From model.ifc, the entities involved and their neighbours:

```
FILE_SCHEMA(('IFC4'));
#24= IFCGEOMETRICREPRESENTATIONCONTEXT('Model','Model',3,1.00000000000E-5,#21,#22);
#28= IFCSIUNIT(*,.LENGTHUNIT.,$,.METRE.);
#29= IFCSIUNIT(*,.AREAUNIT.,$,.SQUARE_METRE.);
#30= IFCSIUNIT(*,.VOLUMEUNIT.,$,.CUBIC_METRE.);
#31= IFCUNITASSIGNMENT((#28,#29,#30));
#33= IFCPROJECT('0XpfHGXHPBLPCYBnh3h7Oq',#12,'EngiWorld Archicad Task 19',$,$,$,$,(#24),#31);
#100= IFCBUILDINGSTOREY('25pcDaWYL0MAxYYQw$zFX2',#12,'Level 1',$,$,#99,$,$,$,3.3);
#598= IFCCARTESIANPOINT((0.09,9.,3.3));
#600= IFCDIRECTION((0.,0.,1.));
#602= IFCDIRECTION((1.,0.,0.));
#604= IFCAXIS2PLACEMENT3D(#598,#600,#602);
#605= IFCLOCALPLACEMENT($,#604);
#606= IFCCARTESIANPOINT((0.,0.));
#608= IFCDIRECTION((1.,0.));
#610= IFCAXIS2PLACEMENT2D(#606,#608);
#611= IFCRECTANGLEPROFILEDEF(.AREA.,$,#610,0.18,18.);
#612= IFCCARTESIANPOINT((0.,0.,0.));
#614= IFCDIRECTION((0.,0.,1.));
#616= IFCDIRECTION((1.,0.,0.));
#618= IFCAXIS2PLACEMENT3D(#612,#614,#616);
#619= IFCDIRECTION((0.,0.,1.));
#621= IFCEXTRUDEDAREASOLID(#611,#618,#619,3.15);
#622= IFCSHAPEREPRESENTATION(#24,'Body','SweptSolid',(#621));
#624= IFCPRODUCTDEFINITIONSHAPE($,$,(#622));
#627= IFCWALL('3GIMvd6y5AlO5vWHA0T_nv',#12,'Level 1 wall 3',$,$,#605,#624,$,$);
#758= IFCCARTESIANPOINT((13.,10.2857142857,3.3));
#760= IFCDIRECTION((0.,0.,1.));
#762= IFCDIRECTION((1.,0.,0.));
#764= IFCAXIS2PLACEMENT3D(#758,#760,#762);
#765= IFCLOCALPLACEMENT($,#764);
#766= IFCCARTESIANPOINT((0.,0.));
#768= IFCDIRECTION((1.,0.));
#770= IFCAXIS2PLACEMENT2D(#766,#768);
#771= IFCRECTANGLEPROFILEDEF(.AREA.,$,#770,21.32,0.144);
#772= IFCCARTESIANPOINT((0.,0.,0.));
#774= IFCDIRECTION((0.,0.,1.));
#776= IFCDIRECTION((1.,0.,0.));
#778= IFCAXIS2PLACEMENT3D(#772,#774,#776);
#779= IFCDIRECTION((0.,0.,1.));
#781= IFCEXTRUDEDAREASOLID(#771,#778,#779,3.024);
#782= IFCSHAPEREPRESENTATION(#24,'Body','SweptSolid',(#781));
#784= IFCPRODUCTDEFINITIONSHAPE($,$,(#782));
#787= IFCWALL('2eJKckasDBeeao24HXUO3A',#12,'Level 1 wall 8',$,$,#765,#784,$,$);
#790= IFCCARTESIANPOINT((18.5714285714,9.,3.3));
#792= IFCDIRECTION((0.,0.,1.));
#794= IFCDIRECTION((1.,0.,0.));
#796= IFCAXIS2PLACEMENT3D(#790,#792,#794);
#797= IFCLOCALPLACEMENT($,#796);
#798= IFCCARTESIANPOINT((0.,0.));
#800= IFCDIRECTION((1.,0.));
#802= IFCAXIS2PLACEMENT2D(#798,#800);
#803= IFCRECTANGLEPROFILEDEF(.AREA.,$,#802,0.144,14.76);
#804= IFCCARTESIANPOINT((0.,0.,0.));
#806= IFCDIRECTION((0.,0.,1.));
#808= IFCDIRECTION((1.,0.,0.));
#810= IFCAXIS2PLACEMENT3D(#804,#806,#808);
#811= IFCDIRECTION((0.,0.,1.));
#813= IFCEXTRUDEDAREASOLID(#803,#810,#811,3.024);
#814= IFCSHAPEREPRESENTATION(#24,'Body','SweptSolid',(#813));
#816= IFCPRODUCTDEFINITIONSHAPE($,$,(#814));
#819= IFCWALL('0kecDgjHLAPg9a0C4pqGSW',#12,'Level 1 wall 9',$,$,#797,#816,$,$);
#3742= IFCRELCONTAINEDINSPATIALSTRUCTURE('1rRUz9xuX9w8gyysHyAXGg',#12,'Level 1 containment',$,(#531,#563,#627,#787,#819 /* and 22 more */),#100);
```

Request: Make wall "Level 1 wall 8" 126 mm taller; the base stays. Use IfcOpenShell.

```python
import ifcopenshell
import ifcopenshell.geom
import ifcopenshell.util.shape
import ifcopenshell.util.unit

model = ifcopenshell.open("model.ifc")
unit_scale = ifcopenshell.util.unit.calculate_unit_scale(model)
settings = ifcopenshell.geom.settings()


def volume(element):
    """Net volume in cubic metres, openings subtracted."""
    shape = ifcopenshell.geom.create_shape(settings, element)
    return ifcopenshell.util.shape.get_volume(shape.geometry)


wall = model.by_guid("2eJKckasDBeeao24HXUO3A")
before = volume(wall)

body = next(r for r in wall.Representation.Representations if r.RepresentationIdentifier == "Body")
solid = body.Items[0]
old_height = solid.Depth
solid.Depth += 0.126 / unit_scale
after = volume(wall)

print(f"height {old_height:g} -> {solid.Depth:g}, volume {before:.3f} -> {after:.3f} m3")

model.write("model_v2.ifc")
```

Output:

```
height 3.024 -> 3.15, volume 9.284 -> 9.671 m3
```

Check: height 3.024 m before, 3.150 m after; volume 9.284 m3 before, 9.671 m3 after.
